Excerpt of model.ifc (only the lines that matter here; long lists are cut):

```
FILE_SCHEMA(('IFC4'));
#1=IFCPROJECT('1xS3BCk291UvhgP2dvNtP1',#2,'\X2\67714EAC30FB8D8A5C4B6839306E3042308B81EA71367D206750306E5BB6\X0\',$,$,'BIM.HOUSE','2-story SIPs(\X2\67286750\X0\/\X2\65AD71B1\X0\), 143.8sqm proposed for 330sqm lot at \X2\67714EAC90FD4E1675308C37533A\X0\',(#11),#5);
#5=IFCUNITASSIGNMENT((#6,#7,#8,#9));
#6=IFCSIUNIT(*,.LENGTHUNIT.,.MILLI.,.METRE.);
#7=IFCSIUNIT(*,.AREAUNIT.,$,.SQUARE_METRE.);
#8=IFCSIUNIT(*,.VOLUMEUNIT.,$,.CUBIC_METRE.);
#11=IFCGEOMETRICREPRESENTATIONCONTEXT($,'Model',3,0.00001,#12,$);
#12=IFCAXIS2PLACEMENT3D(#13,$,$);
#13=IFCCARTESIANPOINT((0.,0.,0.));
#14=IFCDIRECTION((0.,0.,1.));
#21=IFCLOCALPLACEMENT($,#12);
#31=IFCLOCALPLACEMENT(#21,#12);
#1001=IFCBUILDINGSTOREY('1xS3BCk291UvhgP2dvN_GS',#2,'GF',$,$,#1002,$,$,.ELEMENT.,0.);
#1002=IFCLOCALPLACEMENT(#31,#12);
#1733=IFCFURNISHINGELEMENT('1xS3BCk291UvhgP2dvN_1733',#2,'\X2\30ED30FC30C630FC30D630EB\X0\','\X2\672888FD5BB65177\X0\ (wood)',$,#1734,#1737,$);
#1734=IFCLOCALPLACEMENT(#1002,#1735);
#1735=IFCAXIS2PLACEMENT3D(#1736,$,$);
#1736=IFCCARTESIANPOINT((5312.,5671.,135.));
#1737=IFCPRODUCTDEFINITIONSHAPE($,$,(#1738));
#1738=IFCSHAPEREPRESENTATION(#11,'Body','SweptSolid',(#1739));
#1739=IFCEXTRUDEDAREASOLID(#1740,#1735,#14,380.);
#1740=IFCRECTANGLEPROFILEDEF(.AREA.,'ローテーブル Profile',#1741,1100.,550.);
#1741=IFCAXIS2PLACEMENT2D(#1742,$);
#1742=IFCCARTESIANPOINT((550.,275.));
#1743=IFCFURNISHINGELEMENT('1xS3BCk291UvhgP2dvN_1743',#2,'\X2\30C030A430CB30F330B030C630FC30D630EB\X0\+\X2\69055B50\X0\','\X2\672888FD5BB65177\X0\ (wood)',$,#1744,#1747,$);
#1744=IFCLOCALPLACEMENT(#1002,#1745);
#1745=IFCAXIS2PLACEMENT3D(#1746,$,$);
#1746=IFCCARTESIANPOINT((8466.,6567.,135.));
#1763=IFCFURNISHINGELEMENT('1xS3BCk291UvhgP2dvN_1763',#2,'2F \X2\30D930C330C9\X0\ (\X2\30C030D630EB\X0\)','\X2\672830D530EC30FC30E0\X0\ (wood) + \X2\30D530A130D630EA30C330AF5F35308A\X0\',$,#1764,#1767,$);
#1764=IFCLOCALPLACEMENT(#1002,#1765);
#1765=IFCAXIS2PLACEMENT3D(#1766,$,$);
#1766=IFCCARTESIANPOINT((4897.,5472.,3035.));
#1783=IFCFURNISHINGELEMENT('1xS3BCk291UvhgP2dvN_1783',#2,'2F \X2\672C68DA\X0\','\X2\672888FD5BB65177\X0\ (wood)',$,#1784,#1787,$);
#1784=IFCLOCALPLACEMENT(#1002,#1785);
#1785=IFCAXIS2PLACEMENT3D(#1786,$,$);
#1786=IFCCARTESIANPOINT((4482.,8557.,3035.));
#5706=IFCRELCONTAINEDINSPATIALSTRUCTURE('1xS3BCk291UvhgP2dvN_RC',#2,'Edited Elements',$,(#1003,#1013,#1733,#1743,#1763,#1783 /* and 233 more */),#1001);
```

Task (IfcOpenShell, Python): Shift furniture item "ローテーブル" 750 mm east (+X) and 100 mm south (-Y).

```python
import ifcopenshell
import ifcopenshell.api.geometry
import ifcopenshell.util.placement
import ifcopenshell.util.unit

model = ifcopenshell.open("model.ifc")
unit_scale = ifcopenshell.util.unit.calculate_unit_scale(model)

item = model.by_guid("1xS3BCk291UvhgP2dvN_1733")
matrix = ifcopenshell.util.placement.get_local_placement(item.ObjectPlacement)
matrix[0, 3] += 0.75 / unit_scale
matrix[1, 3] -= 0.1 / unit_scale
ifcopenshell.api.geometry.edit_object_placement(model, product=item, matrix=matrix, is_si=False)

print(ifcopenshell.util.placement.get_local_placement(item.ObjectPlacement).round(3) + 0.0)

model.write("model_v2.ifc")
```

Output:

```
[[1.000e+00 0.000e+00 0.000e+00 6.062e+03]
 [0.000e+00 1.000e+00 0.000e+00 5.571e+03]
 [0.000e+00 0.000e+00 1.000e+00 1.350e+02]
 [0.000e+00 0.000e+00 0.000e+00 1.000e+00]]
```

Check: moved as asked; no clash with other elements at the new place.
